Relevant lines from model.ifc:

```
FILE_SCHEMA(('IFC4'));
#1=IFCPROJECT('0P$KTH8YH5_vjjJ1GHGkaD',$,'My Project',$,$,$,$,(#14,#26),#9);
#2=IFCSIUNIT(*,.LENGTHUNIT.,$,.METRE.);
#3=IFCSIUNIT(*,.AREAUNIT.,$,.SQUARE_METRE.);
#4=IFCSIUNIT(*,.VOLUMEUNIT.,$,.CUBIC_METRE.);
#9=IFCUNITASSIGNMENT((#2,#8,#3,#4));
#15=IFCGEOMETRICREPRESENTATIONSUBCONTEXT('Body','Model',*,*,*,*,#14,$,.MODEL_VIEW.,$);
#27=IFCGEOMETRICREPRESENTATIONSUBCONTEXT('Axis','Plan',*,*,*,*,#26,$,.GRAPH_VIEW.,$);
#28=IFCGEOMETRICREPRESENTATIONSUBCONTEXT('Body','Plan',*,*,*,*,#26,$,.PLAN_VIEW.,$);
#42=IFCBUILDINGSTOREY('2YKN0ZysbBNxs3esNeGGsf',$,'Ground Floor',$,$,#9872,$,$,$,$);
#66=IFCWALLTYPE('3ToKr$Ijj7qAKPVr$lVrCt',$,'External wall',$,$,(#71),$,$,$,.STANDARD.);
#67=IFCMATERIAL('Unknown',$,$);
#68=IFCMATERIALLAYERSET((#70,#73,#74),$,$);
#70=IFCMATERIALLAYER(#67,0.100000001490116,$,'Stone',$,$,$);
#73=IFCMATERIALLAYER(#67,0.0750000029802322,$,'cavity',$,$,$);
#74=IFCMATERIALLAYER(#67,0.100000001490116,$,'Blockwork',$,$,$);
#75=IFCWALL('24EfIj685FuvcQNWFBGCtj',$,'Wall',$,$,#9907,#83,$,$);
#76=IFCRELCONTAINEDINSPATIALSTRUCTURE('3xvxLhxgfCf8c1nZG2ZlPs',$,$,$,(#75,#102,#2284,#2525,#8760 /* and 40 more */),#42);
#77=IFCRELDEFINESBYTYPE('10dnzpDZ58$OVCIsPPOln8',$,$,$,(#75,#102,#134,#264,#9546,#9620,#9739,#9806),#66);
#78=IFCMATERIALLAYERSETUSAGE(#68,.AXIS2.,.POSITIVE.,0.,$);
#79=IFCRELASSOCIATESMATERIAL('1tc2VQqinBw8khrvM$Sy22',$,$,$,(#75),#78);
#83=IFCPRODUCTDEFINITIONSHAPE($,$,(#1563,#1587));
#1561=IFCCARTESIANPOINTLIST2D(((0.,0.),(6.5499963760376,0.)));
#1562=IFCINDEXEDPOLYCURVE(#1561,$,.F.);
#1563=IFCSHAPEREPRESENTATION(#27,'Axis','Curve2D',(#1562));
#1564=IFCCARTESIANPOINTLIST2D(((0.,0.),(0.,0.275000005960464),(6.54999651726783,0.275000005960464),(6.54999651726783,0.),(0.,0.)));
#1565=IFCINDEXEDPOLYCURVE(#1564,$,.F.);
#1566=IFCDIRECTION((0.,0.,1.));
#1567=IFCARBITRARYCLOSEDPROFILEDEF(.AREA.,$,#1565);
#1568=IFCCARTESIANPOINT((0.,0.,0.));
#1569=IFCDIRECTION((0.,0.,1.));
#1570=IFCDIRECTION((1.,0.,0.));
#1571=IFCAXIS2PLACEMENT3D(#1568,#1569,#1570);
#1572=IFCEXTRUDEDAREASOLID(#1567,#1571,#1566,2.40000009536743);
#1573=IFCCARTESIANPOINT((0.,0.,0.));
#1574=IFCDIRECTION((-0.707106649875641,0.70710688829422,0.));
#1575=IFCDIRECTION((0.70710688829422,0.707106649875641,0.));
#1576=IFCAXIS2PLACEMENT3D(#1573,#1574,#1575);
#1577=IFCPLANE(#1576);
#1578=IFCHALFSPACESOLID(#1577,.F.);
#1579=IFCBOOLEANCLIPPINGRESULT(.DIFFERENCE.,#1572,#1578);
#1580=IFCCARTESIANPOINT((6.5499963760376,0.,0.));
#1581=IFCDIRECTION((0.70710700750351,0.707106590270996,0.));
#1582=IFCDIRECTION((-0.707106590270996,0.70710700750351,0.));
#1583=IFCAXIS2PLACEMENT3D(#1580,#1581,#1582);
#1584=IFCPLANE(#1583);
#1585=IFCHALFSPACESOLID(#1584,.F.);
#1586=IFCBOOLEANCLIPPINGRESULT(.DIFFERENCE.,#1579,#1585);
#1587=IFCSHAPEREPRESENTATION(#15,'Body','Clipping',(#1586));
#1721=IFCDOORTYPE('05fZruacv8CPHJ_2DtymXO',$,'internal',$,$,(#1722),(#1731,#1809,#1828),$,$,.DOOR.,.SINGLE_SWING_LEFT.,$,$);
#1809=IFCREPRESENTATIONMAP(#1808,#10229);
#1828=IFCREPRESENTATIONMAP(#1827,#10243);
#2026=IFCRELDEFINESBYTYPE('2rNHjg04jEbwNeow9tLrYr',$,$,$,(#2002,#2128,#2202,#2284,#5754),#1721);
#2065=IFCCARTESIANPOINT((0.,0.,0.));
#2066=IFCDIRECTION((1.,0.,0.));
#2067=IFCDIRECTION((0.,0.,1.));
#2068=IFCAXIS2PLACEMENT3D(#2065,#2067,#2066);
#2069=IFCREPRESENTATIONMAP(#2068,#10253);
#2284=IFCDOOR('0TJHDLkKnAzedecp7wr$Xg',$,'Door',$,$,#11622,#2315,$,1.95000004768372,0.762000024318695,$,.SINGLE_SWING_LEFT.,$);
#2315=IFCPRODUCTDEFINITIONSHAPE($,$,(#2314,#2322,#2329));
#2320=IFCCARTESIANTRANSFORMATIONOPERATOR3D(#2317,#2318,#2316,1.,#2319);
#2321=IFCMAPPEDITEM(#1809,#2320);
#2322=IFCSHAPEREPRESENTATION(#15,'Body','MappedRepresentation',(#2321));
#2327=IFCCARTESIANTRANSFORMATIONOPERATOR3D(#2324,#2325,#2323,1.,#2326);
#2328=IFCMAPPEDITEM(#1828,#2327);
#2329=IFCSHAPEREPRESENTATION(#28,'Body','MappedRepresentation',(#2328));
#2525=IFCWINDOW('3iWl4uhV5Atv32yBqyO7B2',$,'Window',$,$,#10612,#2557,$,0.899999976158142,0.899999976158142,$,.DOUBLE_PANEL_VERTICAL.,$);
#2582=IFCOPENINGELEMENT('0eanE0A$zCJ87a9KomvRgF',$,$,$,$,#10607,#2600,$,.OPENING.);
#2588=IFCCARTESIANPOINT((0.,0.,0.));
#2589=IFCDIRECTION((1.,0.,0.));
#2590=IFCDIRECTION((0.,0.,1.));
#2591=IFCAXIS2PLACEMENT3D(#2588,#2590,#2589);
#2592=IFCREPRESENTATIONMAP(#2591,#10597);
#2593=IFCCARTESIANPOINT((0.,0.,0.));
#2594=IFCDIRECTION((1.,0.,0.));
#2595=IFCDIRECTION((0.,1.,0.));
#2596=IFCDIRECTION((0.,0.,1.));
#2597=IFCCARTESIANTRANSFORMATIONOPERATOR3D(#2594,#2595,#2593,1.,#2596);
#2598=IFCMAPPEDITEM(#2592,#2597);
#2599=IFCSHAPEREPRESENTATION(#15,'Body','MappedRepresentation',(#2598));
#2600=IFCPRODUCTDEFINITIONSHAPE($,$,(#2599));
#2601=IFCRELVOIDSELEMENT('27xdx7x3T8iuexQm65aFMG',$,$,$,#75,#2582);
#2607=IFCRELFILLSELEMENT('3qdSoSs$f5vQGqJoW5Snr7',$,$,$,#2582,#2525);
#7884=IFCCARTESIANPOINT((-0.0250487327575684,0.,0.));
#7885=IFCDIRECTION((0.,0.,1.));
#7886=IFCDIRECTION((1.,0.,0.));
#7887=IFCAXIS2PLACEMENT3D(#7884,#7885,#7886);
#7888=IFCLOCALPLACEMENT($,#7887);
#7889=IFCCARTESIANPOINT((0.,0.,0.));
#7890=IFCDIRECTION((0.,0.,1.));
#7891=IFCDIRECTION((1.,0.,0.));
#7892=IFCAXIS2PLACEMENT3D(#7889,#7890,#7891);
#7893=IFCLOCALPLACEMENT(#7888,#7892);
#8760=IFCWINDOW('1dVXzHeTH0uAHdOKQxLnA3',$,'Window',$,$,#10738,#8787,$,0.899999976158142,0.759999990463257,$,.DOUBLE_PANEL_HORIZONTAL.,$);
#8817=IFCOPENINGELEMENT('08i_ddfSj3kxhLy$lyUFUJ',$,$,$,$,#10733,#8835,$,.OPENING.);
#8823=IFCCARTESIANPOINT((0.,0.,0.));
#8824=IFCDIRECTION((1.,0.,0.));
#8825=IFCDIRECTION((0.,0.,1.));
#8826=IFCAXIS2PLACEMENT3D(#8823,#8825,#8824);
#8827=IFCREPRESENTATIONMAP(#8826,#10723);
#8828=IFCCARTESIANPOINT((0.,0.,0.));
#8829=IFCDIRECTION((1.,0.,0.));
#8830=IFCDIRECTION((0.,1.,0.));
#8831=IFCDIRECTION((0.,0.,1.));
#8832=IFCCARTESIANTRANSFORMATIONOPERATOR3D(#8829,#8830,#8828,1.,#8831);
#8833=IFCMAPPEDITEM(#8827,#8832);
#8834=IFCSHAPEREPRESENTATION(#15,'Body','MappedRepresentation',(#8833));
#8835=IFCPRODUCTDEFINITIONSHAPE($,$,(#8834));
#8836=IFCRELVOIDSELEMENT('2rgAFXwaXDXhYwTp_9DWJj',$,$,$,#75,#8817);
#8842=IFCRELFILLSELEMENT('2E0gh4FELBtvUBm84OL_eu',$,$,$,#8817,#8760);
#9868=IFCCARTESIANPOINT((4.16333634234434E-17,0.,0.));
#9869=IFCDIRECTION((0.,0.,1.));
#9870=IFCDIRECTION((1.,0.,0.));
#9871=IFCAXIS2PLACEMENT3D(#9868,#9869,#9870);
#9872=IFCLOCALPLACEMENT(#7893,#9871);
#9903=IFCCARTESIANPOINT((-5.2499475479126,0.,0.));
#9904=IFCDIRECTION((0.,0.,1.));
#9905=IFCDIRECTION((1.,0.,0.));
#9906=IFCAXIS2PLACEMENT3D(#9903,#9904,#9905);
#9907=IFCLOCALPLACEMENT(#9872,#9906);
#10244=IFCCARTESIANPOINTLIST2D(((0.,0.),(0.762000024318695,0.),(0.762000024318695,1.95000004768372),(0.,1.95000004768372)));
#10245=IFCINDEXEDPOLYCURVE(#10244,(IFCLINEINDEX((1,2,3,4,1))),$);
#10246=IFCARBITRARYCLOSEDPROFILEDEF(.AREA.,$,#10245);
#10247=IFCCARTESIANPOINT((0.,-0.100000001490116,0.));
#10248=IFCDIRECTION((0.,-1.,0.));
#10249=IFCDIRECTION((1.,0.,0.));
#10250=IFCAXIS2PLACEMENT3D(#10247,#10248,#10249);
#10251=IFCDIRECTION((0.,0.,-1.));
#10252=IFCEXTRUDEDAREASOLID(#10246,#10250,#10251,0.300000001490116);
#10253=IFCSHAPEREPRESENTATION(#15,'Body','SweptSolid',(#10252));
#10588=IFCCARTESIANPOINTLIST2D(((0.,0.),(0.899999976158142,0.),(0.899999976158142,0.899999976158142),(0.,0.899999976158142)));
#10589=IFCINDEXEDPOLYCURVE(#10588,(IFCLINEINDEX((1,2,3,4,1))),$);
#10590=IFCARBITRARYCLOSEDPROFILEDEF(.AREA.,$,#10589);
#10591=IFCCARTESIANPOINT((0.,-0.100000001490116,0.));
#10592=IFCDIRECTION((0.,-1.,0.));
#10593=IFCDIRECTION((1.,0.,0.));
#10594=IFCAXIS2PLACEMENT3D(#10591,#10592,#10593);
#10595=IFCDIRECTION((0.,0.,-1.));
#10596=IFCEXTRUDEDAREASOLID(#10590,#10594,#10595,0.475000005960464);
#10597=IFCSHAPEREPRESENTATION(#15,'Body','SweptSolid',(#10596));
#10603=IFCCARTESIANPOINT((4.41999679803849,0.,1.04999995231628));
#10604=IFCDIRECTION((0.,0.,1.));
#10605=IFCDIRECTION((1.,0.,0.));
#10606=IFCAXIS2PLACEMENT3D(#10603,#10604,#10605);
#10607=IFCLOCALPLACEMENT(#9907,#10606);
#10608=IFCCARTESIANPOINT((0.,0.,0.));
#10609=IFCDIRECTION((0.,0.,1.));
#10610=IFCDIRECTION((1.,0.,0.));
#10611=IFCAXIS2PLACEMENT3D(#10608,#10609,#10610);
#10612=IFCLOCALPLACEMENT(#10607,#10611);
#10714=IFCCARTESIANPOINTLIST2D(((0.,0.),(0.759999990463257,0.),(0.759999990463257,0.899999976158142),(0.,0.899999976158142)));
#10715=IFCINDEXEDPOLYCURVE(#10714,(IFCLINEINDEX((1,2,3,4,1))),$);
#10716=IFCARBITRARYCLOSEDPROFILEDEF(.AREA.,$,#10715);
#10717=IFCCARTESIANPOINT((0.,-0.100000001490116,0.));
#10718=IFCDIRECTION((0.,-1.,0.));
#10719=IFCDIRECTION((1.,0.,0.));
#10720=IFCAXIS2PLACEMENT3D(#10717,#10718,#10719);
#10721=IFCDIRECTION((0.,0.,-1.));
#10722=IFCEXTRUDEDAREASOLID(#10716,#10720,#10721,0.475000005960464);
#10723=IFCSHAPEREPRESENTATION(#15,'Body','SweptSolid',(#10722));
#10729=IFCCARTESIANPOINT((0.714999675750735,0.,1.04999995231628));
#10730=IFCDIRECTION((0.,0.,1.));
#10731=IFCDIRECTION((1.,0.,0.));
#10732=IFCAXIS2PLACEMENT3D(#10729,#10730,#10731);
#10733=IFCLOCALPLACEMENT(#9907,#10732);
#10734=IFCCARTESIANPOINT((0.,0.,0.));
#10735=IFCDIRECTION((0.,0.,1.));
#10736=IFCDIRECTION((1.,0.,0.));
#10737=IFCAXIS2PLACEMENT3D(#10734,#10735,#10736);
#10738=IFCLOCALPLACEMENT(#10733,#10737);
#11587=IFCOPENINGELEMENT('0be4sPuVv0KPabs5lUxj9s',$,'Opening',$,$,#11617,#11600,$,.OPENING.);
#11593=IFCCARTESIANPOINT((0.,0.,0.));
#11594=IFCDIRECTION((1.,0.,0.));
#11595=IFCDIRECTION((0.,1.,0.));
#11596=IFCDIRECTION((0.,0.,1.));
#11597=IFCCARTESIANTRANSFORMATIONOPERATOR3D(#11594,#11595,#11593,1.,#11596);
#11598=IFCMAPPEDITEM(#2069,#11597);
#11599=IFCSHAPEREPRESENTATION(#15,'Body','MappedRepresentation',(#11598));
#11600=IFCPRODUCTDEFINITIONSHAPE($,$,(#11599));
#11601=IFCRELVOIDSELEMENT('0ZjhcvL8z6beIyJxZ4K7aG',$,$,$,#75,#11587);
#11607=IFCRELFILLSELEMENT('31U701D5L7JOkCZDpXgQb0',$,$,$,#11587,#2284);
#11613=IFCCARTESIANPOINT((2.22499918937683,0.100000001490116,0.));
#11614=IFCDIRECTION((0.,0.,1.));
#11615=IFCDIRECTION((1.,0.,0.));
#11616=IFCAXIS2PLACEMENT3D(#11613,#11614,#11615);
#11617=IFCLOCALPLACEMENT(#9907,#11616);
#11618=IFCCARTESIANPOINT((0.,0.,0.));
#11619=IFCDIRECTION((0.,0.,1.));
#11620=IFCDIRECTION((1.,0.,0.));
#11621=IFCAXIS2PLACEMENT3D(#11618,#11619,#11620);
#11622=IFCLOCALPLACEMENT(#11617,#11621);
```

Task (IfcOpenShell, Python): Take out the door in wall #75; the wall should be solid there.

```python
import ifcopenshell
import ifcopenshell.api.feature
import ifcopenshell.api.root
import ifcopenshell.geom
import ifcopenshell.util.shape

model = ifcopenshell.open("model.ifc")
settings = ifcopenshell.geom.settings()


def volume(element):
    """Net volume in cubic metres, openings subtracted."""
    shape = ifcopenshell.geom.create_shape(settings, element)
    return ifcopenshell.util.shape.get_volume(shape.geometry)


door = model.by_guid("0TJHDLkKnAzedecp7wr$Xg")
opening = door.FillsVoids[0].RelatingOpeningElement
wall = opening.VoidsElements[0].RelatingBuildingElement
before = volume(wall)

ifcopenshell.api.root.remove_product(model, product=door)
ifcopenshell.api.feature.remove_feature(model, feature=opening)

after = volume(wall)

print(f"wall volume {before:.3f} -> {after:.3f} m3")

model.write("model_updated.ifc")
```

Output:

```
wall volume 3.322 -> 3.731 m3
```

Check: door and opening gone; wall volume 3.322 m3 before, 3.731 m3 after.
